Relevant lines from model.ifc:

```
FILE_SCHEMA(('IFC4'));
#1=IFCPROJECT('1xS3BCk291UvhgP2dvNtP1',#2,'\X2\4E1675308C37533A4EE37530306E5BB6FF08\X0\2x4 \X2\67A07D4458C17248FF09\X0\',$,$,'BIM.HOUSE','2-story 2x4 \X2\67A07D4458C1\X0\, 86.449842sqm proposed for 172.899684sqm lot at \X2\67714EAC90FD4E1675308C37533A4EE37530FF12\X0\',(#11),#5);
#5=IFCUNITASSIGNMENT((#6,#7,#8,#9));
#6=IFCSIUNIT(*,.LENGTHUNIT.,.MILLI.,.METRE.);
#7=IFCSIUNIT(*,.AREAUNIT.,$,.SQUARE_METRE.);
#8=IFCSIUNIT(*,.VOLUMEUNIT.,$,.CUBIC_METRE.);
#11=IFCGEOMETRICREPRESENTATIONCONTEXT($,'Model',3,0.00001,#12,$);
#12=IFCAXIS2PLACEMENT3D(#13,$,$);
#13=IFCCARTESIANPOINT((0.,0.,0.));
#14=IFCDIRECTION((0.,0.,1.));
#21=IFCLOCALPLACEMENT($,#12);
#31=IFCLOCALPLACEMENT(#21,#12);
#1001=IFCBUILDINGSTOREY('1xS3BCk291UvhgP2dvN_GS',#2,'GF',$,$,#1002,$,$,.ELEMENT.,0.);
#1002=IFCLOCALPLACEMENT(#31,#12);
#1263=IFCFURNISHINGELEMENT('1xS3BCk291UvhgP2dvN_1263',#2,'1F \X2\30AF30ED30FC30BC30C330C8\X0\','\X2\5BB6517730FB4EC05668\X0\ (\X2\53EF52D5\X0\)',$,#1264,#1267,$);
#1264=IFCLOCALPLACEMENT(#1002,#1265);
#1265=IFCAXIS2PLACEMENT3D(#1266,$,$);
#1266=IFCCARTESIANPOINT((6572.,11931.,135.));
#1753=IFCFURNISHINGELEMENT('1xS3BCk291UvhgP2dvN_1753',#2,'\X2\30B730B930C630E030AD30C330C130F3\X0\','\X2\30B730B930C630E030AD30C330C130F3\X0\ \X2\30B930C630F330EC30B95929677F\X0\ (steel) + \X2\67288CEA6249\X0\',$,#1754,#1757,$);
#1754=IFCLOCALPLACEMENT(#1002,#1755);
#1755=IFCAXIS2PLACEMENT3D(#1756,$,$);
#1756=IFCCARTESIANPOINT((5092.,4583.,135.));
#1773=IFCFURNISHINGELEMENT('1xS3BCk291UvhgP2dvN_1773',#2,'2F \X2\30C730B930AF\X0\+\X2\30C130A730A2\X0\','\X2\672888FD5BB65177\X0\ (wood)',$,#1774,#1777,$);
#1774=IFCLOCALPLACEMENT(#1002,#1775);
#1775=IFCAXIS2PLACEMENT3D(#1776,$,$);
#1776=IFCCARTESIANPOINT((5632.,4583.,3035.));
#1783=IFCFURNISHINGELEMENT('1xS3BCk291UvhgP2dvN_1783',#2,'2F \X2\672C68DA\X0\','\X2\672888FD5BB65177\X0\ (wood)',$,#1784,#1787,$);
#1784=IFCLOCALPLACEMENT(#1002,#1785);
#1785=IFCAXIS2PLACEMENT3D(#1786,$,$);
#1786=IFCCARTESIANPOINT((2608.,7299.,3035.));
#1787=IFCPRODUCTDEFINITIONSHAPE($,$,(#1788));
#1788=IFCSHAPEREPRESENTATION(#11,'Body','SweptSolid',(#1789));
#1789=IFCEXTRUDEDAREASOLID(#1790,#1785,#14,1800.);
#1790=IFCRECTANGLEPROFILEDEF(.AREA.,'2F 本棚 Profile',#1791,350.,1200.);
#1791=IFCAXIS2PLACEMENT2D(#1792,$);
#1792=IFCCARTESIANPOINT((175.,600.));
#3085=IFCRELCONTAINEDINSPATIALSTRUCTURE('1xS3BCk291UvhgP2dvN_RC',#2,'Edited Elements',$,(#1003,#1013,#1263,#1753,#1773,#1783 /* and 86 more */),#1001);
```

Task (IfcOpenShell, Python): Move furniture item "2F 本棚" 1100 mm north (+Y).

```python
import ifcopenshell
import ifcopenshell.api.geometry
import ifcopenshell.util.placement
import ifcopenshell.util.unit

model = ifcopenshell.open("model.ifc")
unit_scale = ifcopenshell.util.unit.calculate_unit_scale(model)

item = model.by_guid("1xS3BCk291UvhgP2dvN_1783")
matrix = ifcopenshell.util.placement.get_local_placement(item.ObjectPlacement)
matrix[1, 3] += 1.1 / unit_scale
ifcopenshell.api.geometry.edit_object_placement(model, product=item, matrix=matrix, is_si=False)

print(ifcopenshell.util.placement.get_local_placement(item.ObjectPlacement).round(3) + 0.0)

model.write("model_v2.ifc")
```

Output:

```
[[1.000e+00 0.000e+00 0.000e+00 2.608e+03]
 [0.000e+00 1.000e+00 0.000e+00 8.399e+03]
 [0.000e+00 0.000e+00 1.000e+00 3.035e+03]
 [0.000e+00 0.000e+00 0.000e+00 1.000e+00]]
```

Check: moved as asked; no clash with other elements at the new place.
